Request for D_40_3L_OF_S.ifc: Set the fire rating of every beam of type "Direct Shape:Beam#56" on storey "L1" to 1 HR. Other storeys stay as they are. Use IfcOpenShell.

First a look at what the model holds.

```python
import ifcopenshell
import ifcopenshell.util.element

model = ifcopenshell.open("D_40_3L_OF_S.ifc")
print(model.schema)
storey = next(s for s in model.by_type("IfcBuildingStorey") if s.Name == "L1")
beams = [e for e in ifcopenshell.util.element.get_decomposition(storey) if e.is_a("IfcBeam")]
seen = {}
for e in beams:
    element_type = ifcopenshell.util.element.get_type(e)
    key = (element_type.Name if element_type != e and element_type else None, ifcopenshell.util.element.get_pset(e, "Pset_BeamCommon", "FireRating"))
    seen[key] = seen.get(key, 0) + 1
for (name, value), count in sorted(seen.items(), key=str):
    print(count, "x", name, "|", value)
```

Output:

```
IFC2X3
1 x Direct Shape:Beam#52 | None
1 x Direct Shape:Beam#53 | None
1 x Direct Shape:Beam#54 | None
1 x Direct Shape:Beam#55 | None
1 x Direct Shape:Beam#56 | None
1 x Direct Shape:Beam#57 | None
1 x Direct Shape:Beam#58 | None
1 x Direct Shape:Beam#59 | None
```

```python
import ifcopenshell
import ifcopenshell.api.pset
import ifcopenshell.util.element

model = ifcopenshell.open("D_40_3L_OF_S.ifc")

storey = next(s for s in model.by_type("IfcBuildingStorey") if s.Name == "L1")
beams = [e for e in ifcopenshell.util.element.get_decomposition(storey) if e.is_a("IfcBeam")]

count = 0
for e in beams:
    element_type = ifcopenshell.util.element.get_type(e)
    if element_type in (None, e) or element_type.Name != "Direct Shape:Beam#56":
        continue
    # add_pset returns the element's existing set when there is one.
    pset = ifcopenshell.api.pset.add_pset(model, product=e, name="Pset_BeamCommon")
    ifcopenshell.api.pset.edit_pset(model, pset=pset, properties={"FireRating": "1 HR"})
    count += 1

print(count, "beams updated")

model.write("D_40_3L_OF_S_updated.ifc")
```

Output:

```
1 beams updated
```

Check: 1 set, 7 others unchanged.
